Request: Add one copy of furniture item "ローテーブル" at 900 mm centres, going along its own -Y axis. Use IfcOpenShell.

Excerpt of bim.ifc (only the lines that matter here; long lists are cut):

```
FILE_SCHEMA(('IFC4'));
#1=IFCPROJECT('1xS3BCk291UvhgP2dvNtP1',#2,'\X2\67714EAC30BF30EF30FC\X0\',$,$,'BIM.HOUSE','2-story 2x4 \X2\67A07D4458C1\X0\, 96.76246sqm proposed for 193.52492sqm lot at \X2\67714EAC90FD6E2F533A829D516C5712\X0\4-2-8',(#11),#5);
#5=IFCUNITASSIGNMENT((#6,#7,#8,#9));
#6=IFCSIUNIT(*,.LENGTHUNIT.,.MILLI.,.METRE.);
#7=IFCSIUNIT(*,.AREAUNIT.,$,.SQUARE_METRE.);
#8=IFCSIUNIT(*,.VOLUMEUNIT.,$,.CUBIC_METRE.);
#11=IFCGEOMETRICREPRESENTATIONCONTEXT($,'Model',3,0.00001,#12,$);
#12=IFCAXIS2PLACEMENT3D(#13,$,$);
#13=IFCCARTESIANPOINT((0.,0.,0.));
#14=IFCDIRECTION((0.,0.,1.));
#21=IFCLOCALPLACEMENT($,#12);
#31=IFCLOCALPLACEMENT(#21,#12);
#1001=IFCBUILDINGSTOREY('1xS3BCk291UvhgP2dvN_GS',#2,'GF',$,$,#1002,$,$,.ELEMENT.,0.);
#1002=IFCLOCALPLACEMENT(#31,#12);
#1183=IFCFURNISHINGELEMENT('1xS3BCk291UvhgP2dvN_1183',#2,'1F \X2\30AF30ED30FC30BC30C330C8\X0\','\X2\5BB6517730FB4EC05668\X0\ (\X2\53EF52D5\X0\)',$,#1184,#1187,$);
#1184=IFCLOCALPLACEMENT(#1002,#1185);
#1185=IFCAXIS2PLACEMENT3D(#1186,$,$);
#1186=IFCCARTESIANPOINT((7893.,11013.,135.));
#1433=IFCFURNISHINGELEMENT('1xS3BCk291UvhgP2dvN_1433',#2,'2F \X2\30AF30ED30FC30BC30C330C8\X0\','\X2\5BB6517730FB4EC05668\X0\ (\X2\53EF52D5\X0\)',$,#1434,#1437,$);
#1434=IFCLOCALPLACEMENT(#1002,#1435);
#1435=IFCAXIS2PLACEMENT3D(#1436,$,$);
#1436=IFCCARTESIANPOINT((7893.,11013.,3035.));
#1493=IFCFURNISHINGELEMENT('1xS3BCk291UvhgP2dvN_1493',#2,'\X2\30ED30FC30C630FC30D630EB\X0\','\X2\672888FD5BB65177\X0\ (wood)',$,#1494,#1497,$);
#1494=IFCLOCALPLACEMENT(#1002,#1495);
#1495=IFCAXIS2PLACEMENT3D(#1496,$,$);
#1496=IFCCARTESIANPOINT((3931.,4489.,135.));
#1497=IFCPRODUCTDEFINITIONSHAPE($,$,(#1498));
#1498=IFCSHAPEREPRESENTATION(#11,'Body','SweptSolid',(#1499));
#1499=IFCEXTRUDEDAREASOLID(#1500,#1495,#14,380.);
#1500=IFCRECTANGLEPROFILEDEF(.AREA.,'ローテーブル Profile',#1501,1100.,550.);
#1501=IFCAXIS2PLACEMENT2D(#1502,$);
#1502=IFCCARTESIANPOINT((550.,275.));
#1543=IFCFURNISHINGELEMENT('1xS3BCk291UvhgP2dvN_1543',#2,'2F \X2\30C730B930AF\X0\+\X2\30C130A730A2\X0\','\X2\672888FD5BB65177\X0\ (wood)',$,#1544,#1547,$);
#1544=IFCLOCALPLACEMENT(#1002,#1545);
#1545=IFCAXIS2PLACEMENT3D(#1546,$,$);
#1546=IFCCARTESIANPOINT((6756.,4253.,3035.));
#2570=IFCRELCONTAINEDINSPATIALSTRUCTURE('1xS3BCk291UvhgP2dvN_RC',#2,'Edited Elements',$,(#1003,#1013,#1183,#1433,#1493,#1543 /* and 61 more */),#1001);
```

```python
import ifcopenshell
import ifcopenshell.api.geometry
import ifcopenshell.api.root
import ifcopenshell.util.element
import ifcopenshell.util.placement

model = ifcopenshell.open("bim.ifc")


def reuse_history(source, copy):
    """copy_class also copies each property set's owner history, people and application; keep the originals."""
    for rel in copy.IsDefinedBy:
        if rel.is_a("IfcRelDefinesByProperties") and (history := rel.RelatingPropertyDefinition.OwnerHistory):
            rel.RelatingPropertyDefinition.OwnerHistory = source.OwnerHistory
            ifcopenshell.util.element.remove_deep2(model, history)


source = model.by_guid("1xS3BCk291UvhgP2dvN_1493")
base = ifcopenshell.util.placement.get_local_placement(source.ObjectPlacement)
step = -base[:3, 1] * 900.0

for i in range(1, 2):
    copy = ifcopenshell.api.root.copy_class(model, product=source)
    copy.Representation = ifcopenshell.util.element.copy_deep(
        model, source.Representation, exclude=["IfcGeometricRepresentationContext", "IfcRepresentationMap"]
    )
    reuse_history(source, copy)
    matrix = base.copy()
    matrix[:3, 3] += i * step
    print("added at", matrix[:3, 3].round(3) + 0.0)
    ifcopenshell.api.geometry.edit_object_placement(model, product=copy, matrix=matrix, is_si=False)

model.write("bim_rev.ifc")
```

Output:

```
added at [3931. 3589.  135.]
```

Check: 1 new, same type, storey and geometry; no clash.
